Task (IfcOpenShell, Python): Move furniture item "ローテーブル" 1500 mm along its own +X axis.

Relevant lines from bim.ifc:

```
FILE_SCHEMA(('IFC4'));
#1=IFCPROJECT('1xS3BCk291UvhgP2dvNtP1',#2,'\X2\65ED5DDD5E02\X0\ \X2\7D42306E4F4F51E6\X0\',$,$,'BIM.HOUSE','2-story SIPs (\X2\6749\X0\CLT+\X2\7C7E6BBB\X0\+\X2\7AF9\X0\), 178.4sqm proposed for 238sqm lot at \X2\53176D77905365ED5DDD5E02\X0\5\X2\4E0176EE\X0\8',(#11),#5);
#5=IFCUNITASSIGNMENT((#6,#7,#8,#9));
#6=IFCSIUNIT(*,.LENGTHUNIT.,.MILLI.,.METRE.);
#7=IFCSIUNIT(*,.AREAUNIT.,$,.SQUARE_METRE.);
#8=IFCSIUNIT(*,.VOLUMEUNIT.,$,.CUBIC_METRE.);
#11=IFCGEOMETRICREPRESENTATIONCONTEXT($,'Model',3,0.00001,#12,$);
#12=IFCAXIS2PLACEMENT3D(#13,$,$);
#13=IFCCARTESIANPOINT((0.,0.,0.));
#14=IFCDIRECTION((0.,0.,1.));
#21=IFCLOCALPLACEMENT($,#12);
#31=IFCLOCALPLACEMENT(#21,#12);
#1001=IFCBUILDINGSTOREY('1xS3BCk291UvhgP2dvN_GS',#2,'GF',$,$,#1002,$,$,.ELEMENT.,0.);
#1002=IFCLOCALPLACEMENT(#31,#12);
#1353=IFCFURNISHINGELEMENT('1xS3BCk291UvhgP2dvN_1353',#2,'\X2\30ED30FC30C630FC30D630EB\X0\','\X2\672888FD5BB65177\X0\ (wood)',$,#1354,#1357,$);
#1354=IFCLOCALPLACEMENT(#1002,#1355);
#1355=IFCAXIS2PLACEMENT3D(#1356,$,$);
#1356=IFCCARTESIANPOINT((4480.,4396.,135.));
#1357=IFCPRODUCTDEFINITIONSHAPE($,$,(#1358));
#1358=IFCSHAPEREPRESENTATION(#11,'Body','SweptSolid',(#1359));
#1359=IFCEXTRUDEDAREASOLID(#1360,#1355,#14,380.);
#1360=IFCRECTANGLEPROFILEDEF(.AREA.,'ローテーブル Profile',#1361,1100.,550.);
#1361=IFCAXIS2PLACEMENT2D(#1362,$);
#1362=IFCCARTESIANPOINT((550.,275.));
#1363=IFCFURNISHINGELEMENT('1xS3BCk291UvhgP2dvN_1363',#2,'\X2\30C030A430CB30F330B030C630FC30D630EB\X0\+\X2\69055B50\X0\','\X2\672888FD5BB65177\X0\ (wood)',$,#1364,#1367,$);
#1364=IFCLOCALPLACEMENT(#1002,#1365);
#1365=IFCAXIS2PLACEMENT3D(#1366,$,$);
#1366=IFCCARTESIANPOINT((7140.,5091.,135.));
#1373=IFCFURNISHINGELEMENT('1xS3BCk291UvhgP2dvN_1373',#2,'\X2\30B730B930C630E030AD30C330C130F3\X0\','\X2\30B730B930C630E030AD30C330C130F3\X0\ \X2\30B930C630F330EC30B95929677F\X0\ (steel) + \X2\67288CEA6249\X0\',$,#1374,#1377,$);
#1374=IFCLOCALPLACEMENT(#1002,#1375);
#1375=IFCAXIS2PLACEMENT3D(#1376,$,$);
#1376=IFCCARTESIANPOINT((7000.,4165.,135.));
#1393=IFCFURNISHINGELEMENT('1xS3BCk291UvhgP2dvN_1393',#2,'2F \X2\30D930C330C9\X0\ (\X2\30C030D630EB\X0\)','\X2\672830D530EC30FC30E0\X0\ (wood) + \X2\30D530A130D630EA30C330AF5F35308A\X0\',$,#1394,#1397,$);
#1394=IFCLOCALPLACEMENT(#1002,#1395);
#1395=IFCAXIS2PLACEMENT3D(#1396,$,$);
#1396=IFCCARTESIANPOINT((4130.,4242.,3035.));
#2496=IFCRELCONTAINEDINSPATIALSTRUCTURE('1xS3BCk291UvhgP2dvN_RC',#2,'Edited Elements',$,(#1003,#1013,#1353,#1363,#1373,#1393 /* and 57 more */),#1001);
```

```python
import ifcopenshell
import ifcopenshell.api.geometry
import ifcopenshell.util.placement
import ifcopenshell.util.unit

model = ifcopenshell.open("bim.ifc")
unit_scale = ifcopenshell.util.unit.calculate_unit_scale(model)

item = model.by_guid("1xS3BCk291UvhgP2dvN_1353")
matrix = ifcopenshell.util.placement.get_local_placement(item.ObjectPlacement)
matrix[:3, 3] += matrix[:3, 0] * 1.5 / unit_scale
ifcopenshell.api.geometry.edit_object_placement(model, product=item, matrix=matrix, is_si=False)

print(ifcopenshell.util.placement.get_local_placement(item.ObjectPlacement).round(3) + 0.0)

model.write("bim_v2.ifc")
```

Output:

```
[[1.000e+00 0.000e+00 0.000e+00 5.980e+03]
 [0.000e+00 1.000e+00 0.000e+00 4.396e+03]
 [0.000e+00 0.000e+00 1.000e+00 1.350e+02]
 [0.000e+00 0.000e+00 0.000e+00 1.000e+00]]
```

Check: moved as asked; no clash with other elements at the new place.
